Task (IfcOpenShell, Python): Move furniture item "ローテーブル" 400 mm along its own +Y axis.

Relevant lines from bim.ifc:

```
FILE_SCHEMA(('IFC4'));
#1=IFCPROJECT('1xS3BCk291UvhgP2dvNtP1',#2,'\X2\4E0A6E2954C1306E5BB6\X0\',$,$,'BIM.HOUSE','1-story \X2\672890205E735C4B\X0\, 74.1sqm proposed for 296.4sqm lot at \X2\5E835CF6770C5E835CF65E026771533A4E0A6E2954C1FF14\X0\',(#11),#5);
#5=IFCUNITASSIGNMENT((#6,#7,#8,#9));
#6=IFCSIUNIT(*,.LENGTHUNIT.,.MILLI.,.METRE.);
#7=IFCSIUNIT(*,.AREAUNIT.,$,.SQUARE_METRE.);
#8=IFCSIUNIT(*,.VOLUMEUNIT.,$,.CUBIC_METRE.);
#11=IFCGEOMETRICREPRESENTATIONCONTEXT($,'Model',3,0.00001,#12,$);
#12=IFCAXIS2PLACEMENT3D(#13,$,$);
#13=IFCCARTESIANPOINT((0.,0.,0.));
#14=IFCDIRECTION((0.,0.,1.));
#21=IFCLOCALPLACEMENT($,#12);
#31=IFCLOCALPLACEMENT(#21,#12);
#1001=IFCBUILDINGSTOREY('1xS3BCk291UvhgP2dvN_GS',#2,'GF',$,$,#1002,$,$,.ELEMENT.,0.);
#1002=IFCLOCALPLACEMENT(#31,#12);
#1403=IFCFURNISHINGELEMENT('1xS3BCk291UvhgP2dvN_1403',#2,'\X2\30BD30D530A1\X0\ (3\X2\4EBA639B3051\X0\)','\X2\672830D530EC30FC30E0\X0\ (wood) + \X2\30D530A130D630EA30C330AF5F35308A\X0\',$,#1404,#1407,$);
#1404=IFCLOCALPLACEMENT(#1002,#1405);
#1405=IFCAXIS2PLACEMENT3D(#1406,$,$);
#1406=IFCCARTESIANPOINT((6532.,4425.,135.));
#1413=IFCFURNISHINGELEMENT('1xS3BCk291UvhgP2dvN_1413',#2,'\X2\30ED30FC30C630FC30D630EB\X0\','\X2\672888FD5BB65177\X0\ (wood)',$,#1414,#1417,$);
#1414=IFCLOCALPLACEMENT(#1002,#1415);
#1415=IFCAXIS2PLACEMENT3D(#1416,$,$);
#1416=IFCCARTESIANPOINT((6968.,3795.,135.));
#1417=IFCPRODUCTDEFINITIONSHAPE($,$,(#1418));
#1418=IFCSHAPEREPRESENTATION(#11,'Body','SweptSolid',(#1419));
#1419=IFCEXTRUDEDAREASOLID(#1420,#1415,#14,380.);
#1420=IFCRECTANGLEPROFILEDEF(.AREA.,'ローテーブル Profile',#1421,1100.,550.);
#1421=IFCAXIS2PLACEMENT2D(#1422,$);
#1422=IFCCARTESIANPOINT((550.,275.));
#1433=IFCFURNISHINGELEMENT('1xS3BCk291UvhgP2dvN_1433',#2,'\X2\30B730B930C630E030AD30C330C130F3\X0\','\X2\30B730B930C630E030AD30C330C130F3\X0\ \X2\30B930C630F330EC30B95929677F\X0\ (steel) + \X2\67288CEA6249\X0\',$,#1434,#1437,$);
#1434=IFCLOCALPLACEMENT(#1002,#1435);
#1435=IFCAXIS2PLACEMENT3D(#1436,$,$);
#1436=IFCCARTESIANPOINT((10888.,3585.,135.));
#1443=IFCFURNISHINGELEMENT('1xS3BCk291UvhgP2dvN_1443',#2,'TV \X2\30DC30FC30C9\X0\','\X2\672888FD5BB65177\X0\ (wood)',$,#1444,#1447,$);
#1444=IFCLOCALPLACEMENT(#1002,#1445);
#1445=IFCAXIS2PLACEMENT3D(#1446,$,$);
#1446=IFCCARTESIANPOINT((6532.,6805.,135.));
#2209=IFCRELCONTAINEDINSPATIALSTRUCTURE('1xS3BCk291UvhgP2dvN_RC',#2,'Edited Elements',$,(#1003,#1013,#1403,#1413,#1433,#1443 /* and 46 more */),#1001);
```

```python
import ifcopenshell
import ifcopenshell.api.geometry
import ifcopenshell.util.placement
import ifcopenshell.util.unit

model = ifcopenshell.open("bim.ifc")
unit_scale = ifcopenshell.util.unit.calculate_unit_scale(model)

item = model.by_guid("1xS3BCk291UvhgP2dvN_1413")
matrix = ifcopenshell.util.placement.get_local_placement(item.ObjectPlacement)
matrix[:3, 3] += matrix[:3, 1] * 0.4 / unit_scale
ifcopenshell.api.geometry.edit_object_placement(model, product=item, matrix=matrix, is_si=False)

print(ifcopenshell.util.placement.get_local_placement(item.ObjectPlacement).round(3) + 0.0)

model.write("bim_edited.ifc")
```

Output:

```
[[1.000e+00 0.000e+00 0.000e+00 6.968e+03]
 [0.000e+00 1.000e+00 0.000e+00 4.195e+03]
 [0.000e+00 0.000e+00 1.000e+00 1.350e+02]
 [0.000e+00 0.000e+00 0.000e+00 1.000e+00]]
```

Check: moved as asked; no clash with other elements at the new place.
